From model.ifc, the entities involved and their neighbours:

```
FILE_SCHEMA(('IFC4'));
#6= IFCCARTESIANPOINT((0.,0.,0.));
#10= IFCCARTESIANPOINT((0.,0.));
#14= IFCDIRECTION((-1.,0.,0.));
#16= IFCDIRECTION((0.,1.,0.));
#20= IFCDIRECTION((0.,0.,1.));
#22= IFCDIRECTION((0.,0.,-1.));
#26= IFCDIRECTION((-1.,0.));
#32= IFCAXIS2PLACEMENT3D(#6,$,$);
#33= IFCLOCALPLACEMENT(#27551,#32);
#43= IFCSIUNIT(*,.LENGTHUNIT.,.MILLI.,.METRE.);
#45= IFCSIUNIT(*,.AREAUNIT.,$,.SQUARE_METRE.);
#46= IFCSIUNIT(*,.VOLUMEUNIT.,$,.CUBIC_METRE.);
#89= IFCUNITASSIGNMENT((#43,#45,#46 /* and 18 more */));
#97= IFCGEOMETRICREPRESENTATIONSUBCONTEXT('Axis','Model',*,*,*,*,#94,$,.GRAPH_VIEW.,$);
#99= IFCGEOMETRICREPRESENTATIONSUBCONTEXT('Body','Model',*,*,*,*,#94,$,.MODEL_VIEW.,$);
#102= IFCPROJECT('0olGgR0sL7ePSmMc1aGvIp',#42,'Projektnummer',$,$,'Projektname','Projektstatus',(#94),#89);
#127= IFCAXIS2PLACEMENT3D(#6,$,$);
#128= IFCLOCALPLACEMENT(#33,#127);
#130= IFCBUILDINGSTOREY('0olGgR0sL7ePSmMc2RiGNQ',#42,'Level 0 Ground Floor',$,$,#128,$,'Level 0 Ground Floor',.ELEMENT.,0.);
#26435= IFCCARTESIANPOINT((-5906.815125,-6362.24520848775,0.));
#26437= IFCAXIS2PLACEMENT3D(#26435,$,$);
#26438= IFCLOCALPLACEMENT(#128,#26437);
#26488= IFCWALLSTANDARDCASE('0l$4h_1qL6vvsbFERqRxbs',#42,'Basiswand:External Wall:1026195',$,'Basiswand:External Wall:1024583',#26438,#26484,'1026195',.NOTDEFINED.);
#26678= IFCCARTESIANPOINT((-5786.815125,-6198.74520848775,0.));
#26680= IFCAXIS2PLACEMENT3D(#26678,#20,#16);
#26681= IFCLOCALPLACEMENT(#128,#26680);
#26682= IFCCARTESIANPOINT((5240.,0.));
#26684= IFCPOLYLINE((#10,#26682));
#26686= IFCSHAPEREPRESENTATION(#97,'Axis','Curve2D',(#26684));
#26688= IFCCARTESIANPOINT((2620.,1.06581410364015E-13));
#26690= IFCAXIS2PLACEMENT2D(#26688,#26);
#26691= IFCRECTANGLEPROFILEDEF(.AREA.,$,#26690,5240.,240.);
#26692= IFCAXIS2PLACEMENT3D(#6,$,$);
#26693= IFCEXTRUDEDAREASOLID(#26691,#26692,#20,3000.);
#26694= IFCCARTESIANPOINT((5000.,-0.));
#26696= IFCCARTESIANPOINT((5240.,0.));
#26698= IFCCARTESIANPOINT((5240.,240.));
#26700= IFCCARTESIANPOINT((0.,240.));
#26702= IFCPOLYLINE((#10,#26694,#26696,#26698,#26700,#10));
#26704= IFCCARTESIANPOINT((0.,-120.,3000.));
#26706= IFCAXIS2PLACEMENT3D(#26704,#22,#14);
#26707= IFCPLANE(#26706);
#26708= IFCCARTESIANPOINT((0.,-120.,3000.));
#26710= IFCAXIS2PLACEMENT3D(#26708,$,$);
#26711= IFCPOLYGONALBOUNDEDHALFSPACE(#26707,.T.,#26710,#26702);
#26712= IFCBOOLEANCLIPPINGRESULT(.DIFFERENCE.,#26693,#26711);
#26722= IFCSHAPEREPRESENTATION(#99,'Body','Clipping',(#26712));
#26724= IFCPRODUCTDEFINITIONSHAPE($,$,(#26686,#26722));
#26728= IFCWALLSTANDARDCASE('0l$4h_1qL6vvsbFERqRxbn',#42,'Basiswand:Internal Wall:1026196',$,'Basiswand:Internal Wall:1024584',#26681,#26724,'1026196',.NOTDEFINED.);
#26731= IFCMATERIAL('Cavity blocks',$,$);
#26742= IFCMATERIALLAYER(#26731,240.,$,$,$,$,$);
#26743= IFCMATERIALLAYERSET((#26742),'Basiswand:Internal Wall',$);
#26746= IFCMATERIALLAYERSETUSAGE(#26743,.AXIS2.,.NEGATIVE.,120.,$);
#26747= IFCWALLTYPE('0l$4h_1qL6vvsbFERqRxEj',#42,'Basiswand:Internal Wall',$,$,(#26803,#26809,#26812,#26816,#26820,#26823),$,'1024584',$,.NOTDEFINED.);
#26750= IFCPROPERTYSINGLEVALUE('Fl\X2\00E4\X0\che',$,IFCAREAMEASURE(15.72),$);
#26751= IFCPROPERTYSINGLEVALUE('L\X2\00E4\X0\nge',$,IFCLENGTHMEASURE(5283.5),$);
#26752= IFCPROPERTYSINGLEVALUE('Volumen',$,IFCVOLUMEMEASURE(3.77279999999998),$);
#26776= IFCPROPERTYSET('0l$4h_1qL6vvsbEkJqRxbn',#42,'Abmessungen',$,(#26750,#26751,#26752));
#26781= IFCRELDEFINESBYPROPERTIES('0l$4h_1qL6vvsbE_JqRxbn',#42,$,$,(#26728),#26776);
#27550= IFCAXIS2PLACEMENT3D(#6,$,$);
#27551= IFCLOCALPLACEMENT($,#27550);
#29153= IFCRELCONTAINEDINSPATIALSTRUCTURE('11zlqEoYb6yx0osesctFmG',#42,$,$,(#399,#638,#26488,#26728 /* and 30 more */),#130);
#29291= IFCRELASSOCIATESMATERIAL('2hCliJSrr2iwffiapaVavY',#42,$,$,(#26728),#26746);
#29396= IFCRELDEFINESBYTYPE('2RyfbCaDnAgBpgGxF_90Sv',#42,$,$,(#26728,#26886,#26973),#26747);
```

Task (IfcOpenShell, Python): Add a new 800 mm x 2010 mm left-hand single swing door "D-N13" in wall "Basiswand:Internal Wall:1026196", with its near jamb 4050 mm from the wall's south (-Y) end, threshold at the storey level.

```python
import numpy as np
import ifcopenshell
import ifcopenshell.api.feature
import ifcopenshell.api.geometry
import ifcopenshell.api.pset
import ifcopenshell.api.root
import ifcopenshell.api.spatial
import ifcopenshell.geom
import ifcopenshell.util.element
import ifcopenshell.util.placement
import ifcopenshell.util.representation
import ifcopenshell.util.shape
import ifcopenshell.util.unit

model = ifcopenshell.open("model.ifc")
unit_scale = ifcopenshell.util.unit.calculate_unit_scale(model)
area_scale = ifcopenshell.util.unit.calculate_unit_scale(model, "AREAUNIT")
volume_scale = ifcopenshell.util.unit.calculate_unit_scale(model, "VOLUMEUNIT")
settings = ifcopenshell.geom.settings()


def volume(element):
    """Net volume in cubic metres, openings subtracted."""
    shape = ifcopenshell.geom.create_shape(settings, element)
    return ifcopenshell.util.shape.get_volume(shape.geometry)


wall = model.by_guid("0l$4h_1qL6vvsbFERqRxbn")
storey = ifcopenshell.util.element.get_container(wall, ifc_class="IfcBuildingStorey")
context = ifcopenshell.util.representation.get_context(model, "Model", "Body", "MODEL_VIEW")
before = volume(wall)

width, height, from_end, sill = 0.8, 2.01, 4.05, 0.0  # metres

# The wall runs along its own X axis, and the end named is its -X end.
wall_shape = ifcopenshell.geom.create_shape(settings, wall)
x, y, z = ifcopenshell.util.shape.get_vertices(wall_shape.geometry).T
start = x.min() + from_end
face, thickness = float(y.min()), float(y.max() - y.min())
wall_matrix = ifcopenshell.util.placement.get_local_placement(wall.ObjectPlacement)
level = ifcopenshell.util.placement.get_local_placement(storey.ObjectPlacement)[2, 3]


def in_wall(x, y):
    """Placement at x, y metres in the wall's axes, at sill height."""
    matrix = wall_matrix.copy()
    matrix[:, 3] = wall_matrix @ np.array([x / unit_scale, y / unit_scale, 0.0, 1.0])
    matrix[2, 3] = level + sill / unit_scale
    return matrix


# Opening: a box that overshoots both wall faces by 50 mm.
opening = ifcopenshell.api.root.create_entity(model, ifc_class="IfcOpeningElement", predefined_type="OPENING")
box = ifcopenshell.api.geometry.add_wall_representation(
    model, context=context, length=width, height=height, thickness=thickness + 0.1
)
ifcopenshell.api.geometry.assign_representation(model, product=opening, representation=box)
ifcopenshell.api.geometry.edit_object_placement(model, product=opening, matrix=in_wall(start, face - 0.05), is_si=False)
ifcopenshell.api.feature.add_feature(model, feature=opening, element=wall)

door = ifcopenshell.api.root.create_entity(model, ifc_class="IfcDoor", name="D-N13", predefined_type="DOOR")
door.OverallWidth, door.OverallHeight = width / unit_scale, height / unit_scale
door.OperationType = "SINGLE_SWING_LEFT"
body = ifcopenshell.api.geometry.add_door_representation(
    model,
    context=context,
    overall_width=door.OverallWidth,
    overall_height=door.OverallHeight,
    operation_type="SINGLE_SWING_LEFT",
    lining_properties={"LiningDepth": thickness / unit_scale, "ThresholdDepth": thickness / unit_scale},
)
ifcopenshell.api.geometry.assign_representation(model, product=door, representation=body)
ifcopenshell.api.spatial.assign_container(model, products=[door], relating_structure=storey)
ifcopenshell.api.feature.add_filling(model, opening=opening, element=door)

# The lining spans the wall, so the door starts at the wall face.
ifcopenshell.api.geometry.edit_object_placement(model, product=door, matrix=in_wall(start, face), is_si=False)

after = volume(wall)

# Update the wall's stored quantities.
pset = model.by_id(ifcopenshell.util.element.get_pset(wall, "Abmessungen", should_inherit=False)["id"])
ifcopenshell.api.pset.edit_pset(model, pset=pset, properties={
    "Fläche": model.create_entity("IfcAreaMeasure", after / thickness / area_scale),
    "Volumen": model.create_entity("IfcVolumeMeasure", after / volume_scale),
})

print(f"wall volume {before:.3f} -> {after:.3f} m3")

model.write("model_updated.ifc")
```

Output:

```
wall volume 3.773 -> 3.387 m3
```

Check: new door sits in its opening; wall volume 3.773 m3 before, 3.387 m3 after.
